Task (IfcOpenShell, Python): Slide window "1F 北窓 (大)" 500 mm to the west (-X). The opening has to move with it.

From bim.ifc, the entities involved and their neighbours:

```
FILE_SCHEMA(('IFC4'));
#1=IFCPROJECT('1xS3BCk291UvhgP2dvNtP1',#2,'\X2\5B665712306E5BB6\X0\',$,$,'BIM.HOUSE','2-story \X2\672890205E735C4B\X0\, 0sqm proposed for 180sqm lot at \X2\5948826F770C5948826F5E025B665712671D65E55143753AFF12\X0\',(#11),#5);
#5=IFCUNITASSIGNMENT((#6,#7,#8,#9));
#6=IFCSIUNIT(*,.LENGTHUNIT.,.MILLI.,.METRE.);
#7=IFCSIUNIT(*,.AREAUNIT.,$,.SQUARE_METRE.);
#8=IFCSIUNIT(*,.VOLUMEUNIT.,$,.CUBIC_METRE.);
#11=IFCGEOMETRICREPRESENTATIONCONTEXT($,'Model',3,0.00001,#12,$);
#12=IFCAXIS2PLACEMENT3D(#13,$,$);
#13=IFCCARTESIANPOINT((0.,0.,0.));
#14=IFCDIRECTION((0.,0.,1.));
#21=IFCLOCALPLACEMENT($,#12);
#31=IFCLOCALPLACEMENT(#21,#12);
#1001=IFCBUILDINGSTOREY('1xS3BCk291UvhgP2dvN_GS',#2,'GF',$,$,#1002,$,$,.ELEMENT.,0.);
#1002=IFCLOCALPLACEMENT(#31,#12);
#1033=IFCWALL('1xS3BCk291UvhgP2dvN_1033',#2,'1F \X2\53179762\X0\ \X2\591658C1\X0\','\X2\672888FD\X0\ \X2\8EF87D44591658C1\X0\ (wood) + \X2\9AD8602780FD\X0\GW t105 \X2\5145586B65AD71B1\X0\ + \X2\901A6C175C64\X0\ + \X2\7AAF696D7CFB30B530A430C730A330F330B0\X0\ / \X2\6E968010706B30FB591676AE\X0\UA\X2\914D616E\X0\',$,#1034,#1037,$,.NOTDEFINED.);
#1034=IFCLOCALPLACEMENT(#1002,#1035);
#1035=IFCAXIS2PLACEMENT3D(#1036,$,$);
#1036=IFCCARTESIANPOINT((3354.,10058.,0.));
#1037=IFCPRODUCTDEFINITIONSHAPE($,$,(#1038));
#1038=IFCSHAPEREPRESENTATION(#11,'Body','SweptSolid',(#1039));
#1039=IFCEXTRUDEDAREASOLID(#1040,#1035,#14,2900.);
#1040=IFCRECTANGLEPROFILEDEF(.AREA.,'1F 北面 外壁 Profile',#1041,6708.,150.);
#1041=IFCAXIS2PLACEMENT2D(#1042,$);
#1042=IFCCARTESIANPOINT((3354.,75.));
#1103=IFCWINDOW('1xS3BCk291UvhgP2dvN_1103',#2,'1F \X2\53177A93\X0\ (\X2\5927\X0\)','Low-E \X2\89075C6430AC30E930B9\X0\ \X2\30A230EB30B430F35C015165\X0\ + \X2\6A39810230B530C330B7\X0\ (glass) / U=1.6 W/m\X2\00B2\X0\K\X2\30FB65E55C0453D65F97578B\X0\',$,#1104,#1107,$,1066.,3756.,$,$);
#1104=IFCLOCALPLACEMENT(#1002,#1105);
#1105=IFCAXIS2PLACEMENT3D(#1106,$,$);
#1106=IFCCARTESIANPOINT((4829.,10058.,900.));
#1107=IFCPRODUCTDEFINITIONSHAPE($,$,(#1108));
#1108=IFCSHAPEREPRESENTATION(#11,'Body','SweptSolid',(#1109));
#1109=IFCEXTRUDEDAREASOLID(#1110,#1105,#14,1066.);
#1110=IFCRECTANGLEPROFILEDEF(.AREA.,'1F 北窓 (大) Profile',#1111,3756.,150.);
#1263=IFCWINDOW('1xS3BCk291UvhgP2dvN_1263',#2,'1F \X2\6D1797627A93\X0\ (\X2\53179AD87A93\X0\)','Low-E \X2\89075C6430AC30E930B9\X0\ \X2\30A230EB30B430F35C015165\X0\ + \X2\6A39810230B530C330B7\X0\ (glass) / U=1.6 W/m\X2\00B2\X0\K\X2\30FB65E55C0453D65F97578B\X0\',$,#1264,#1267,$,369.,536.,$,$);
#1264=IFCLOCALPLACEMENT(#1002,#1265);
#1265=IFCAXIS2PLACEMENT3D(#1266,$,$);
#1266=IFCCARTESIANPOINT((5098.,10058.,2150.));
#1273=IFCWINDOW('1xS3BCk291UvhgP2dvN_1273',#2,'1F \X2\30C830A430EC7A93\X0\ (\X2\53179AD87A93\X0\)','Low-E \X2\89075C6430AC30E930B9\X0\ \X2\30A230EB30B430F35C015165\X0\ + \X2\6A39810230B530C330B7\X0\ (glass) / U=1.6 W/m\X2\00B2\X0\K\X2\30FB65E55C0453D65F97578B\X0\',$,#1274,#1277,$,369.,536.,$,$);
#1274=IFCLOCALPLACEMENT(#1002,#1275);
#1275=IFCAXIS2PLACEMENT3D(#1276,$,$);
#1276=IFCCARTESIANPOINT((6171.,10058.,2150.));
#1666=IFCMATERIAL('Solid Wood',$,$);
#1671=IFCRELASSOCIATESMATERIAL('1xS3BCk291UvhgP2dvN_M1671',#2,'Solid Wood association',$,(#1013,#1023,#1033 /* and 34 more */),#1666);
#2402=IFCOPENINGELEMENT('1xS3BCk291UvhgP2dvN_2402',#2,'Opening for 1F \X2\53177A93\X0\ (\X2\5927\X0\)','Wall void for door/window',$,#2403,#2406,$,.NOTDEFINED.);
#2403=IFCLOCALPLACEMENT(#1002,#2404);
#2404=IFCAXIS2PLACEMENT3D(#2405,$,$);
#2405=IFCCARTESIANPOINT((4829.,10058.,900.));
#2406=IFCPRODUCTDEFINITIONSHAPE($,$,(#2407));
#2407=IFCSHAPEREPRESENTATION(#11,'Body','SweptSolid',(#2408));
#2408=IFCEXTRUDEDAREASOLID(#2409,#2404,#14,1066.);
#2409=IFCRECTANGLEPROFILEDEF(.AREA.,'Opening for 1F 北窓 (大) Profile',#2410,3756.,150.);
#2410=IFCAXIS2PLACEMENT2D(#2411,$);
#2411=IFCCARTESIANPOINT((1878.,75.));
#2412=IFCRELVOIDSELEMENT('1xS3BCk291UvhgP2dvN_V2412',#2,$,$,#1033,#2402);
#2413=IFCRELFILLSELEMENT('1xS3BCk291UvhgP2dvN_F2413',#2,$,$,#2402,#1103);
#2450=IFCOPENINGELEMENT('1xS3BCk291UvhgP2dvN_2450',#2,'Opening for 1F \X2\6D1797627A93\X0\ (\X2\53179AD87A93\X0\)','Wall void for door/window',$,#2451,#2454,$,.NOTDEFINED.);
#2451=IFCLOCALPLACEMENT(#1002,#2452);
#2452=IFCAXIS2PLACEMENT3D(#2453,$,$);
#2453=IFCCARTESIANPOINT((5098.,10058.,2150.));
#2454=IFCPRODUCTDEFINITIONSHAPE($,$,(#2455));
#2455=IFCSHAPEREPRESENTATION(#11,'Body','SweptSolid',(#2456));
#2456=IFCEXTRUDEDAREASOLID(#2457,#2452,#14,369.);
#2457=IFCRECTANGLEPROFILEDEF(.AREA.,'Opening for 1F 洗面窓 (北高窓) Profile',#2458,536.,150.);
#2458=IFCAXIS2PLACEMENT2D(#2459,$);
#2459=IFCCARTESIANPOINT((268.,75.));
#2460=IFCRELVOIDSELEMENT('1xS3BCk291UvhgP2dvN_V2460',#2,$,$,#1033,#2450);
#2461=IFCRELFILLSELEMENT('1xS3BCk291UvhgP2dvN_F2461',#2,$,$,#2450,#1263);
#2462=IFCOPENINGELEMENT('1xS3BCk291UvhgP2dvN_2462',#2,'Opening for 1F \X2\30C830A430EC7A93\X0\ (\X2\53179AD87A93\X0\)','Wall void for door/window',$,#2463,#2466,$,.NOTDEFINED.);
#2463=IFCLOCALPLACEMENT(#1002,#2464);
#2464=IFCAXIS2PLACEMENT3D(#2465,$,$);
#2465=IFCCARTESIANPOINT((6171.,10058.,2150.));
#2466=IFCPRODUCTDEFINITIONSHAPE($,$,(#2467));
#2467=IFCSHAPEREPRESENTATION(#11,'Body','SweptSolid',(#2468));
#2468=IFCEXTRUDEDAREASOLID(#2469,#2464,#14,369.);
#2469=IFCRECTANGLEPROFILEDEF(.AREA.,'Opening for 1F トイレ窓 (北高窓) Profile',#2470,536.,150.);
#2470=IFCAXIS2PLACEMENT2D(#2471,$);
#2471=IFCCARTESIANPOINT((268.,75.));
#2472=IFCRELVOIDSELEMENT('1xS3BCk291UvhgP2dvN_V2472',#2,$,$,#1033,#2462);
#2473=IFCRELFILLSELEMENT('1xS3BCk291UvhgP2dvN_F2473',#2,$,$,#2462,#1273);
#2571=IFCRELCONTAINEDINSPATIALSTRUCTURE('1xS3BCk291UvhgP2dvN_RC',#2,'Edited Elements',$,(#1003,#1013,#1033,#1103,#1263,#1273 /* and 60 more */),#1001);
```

```python
import ifcopenshell
import ifcopenshell.api.geometry
import ifcopenshell.util.placement
import ifcopenshell.util.unit

model = ifcopenshell.open("bim.ifc")
unit_scale = ifcopenshell.util.unit.calculate_unit_scale(model)

window = model.by_guid("1xS3BCk291UvhgP2dvN_1103")
opening = window.FillsVoids[0].RelatingOpeningElement
wall = opening.VoidsElements[0].RelatingBuildingElement

wall_matrix = ifcopenshell.util.placement.get_local_placement(wall.ObjectPlacement)
shift = wall_matrix[:3, 0] * -0.5 / unit_scale
before = ifcopenshell.util.placement.get_local_placement(window.ObjectPlacement)[:3, 3].copy()

# The window is not placed relative to its opening, so move both.
for product in (opening, window):
    matrix = ifcopenshell.util.placement.get_local_placement(product.ObjectPlacement)
    matrix[:3, 3] += shift
    ifcopenshell.api.geometry.edit_object_placement(model, product=product, matrix=matrix, is_si=False)

after = ifcopenshell.util.placement.get_local_placement(window.ObjectPlacement)[:3, 3]
print("window moved by", (after - before).round(3) + 0.0)

model.write("bim_edited.ifc")
```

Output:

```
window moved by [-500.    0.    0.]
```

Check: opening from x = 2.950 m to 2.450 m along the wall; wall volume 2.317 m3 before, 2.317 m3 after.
